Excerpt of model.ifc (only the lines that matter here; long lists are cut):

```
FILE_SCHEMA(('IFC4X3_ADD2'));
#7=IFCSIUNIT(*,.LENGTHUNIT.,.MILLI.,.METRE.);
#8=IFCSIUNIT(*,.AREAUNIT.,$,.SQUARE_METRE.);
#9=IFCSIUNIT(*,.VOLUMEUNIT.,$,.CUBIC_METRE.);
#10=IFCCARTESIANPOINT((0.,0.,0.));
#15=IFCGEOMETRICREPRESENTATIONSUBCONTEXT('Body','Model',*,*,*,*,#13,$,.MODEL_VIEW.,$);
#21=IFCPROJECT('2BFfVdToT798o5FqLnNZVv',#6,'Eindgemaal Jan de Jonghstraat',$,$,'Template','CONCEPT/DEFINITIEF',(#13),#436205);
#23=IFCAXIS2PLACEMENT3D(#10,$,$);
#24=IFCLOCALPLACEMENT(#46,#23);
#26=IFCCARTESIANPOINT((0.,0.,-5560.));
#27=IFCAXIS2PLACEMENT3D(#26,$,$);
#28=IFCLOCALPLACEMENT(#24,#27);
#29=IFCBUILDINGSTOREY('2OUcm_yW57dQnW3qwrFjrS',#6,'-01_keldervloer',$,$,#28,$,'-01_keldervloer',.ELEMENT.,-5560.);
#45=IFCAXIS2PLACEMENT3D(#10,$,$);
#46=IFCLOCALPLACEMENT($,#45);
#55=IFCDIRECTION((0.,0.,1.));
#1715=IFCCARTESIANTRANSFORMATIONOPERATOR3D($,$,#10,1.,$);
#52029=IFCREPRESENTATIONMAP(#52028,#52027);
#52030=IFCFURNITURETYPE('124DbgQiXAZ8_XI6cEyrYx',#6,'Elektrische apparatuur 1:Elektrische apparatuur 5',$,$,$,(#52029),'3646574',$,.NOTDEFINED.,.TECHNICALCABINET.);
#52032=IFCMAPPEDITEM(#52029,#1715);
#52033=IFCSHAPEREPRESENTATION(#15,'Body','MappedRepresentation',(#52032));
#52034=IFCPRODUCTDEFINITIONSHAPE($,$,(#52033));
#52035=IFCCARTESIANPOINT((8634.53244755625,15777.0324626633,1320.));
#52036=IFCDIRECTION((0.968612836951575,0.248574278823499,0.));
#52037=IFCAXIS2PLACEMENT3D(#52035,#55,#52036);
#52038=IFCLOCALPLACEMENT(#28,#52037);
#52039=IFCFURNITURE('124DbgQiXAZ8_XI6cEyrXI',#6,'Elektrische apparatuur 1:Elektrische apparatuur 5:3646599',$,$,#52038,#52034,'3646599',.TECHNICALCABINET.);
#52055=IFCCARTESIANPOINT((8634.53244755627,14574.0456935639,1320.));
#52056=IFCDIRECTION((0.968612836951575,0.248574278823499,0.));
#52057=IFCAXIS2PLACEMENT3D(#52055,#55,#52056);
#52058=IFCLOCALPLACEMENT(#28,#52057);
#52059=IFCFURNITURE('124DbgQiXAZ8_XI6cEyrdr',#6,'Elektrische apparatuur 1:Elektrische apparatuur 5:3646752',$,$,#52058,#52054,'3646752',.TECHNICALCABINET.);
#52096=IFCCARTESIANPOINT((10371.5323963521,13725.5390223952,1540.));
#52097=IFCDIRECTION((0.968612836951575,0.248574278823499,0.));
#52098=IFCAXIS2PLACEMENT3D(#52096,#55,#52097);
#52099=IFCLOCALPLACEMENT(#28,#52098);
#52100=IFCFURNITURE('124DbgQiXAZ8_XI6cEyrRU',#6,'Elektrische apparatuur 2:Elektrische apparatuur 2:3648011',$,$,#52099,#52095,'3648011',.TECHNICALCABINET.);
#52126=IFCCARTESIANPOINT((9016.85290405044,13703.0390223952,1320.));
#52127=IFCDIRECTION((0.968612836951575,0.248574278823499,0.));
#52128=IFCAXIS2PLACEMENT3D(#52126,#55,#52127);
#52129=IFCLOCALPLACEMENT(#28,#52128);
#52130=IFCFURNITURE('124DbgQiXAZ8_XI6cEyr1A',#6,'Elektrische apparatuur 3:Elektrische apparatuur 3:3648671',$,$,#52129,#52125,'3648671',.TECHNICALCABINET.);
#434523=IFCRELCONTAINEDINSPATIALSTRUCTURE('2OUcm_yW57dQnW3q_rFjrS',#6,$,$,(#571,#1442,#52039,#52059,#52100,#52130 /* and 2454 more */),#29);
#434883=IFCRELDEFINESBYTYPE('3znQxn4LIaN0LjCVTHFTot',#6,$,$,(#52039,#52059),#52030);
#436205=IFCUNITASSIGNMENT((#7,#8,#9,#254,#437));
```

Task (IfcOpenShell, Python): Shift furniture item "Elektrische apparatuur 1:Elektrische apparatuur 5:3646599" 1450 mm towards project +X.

```python
import ifcopenshell
import ifcopenshell.api.geometry
import ifcopenshell.util.placement

model = ifcopenshell.open("model.ifc")

item = model.by_id(52039)
matrix = ifcopenshell.util.placement.get_local_placement(item.ObjectPlacement)
matrix[0, 3] += 1450.0
ifcopenshell.api.geometry.edit_object_placement(model, product=item, matrix=matrix, is_si=False)

print(ifcopenshell.util.placement.get_local_placement(item.ObjectPlacement).round(3) + 0.0)

model.write("model_edited.ifc")
```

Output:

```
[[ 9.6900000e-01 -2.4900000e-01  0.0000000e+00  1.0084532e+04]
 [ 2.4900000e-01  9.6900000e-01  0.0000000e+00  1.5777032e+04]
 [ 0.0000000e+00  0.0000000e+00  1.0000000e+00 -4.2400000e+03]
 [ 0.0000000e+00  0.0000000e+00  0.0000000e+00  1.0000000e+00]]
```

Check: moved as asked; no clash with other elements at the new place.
